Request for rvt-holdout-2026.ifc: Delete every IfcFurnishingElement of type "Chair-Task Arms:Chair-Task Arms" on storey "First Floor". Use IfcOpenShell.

First a look at what the model holds.

```python
import ifcopenshell
import ifcopenshell.util.element

model = ifcopenshell.open("rvt-holdout-2026.ifc")
print(model.schema)
storey = next(s for s in model.by_type("IfcBuildingStorey") if s.Name == "First Floor")
furniture = [e for e in ifcopenshell.util.element.get_decomposition(storey) if e.is_a("IfcFurnishingElement")]
seen = {}
for e in furniture:
    element_type = ifcopenshell.util.element.get_type(e)
    name = element_type.Name if element_type not in (None, e) else None
    seen[name] = seen.get(name, 0) + 1
for name, count in sorted(seen.items(), key=str):
    print(count, "x", name)
```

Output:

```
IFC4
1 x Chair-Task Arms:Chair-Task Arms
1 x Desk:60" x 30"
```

```python
import ifcopenshell
import ifcopenshell.api.root
import ifcopenshell.util.element

model = ifcopenshell.open("rvt-holdout-2026.ifc")

storey = next(s for s in model.by_type("IfcBuildingStorey") if s.Name == "First Floor")
furniture = [e for e in ifcopenshell.util.element.get_decomposition(storey) if e.is_a("IfcFurnishingElement")]
targets = [e for e in furniture if (t := ifcopenshell.util.element.get_type(e)) not in (None, e) and t.Name == "Chair-Task Arms:Chair-Task Arms"]

for e in targets:
    ifcopenshell.api.root.remove_product(model, product=e)
print(len(targets), "removed")

model.write("rvt-holdout-2026-out.ifc")
```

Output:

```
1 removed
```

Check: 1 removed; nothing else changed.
